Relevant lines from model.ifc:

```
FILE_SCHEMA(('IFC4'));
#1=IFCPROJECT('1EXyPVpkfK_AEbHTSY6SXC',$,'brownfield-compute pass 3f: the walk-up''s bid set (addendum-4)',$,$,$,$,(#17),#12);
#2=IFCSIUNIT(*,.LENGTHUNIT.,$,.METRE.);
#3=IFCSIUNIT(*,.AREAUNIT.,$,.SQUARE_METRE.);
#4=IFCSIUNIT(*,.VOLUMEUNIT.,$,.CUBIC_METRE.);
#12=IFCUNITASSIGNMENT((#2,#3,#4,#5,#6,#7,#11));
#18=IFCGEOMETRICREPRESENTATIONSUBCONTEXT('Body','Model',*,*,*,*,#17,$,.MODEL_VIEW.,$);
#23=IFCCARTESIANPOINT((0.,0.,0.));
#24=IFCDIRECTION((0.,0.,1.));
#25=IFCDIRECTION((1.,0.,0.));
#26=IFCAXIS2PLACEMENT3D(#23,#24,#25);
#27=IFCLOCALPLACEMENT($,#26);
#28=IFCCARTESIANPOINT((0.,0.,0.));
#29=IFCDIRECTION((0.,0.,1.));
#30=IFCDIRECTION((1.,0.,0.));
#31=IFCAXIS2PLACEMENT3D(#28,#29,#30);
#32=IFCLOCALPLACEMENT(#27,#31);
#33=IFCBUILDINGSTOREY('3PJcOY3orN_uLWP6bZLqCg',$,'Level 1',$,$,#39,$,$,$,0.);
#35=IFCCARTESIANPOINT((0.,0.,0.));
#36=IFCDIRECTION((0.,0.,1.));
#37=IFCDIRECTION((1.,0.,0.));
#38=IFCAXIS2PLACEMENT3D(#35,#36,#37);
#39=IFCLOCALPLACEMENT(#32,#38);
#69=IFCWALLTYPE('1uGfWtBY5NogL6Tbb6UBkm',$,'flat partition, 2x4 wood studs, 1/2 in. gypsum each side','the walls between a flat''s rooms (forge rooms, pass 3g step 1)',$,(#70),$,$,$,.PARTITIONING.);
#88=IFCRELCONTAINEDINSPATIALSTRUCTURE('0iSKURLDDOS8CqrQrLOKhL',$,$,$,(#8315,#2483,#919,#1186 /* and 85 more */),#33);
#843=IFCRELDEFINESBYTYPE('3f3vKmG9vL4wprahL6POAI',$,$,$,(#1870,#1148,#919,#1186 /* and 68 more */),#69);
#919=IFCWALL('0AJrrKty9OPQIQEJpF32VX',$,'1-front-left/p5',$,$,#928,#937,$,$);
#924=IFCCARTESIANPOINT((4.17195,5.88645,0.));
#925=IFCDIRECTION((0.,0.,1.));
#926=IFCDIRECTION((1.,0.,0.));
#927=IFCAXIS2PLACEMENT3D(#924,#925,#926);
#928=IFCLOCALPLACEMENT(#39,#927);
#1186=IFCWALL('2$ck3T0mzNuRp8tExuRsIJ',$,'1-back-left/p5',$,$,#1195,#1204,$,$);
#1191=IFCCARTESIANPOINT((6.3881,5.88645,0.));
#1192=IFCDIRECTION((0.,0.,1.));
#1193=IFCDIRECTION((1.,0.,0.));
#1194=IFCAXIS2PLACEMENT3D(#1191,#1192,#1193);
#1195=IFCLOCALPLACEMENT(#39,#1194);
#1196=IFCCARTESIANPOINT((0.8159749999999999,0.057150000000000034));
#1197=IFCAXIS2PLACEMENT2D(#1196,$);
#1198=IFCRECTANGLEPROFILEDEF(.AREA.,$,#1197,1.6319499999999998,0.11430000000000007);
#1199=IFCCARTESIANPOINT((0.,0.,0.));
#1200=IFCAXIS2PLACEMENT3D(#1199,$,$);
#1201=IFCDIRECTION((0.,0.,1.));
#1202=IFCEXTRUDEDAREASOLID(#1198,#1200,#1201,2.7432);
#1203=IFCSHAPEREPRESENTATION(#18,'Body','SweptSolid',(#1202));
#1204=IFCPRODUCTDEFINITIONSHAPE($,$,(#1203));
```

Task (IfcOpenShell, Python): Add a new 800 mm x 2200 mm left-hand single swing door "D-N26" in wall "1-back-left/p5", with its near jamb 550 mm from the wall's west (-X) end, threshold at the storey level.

```python
import numpy as np
import ifcopenshell
import ifcopenshell.api.feature
import ifcopenshell.api.geometry
import ifcopenshell.api.root
import ifcopenshell.api.spatial
import ifcopenshell.geom
import ifcopenshell.util.element
import ifcopenshell.util.placement
import ifcopenshell.util.representation
import ifcopenshell.util.shape
import ifcopenshell.util.unit

model = ifcopenshell.open("model.ifc")
unit_scale = ifcopenshell.util.unit.calculate_unit_scale(model)
settings = ifcopenshell.geom.settings()


def volume(element):
    """Net volume in cubic metres, openings subtracted."""
    shape = ifcopenshell.geom.create_shape(settings, element)
    return ifcopenshell.util.shape.get_volume(shape.geometry)


wall = model.by_id(1186)
storey = ifcopenshell.util.element.get_container(wall, ifc_class="IfcBuildingStorey")
context = ifcopenshell.util.representation.get_context(model, "Model", "Body", "MODEL_VIEW")
before = volume(wall)

width, height, from_end, sill = 0.8, 2.2, 0.55, 0.0  # metres

# The wall runs along its own X axis, and the end named is its -X end.
wall_shape = ifcopenshell.geom.create_shape(settings, wall)
x, y, z = ifcopenshell.util.shape.get_vertices(wall_shape.geometry).T
start = x.min() + from_end
face, thickness = float(y.min()), float(y.max() - y.min())
wall_matrix = ifcopenshell.util.placement.get_local_placement(wall.ObjectPlacement)
level = ifcopenshell.util.placement.get_local_placement(storey.ObjectPlacement)[2, 3]


def in_wall(x, y):
    """Placement at x, y metres in the wall's axes, at sill height."""
    matrix = wall_matrix.copy()
    matrix[:, 3] = wall_matrix @ np.array([x / unit_scale, y / unit_scale, 0.0, 1.0])
    matrix[2, 3] = level + sill / unit_scale
    return matrix


# Opening: a box that overshoots both wall faces by 50 mm.
opening = ifcopenshell.api.root.create_entity(model, ifc_class="IfcOpeningElement", predefined_type="OPENING")
box = ifcopenshell.api.geometry.add_wall_representation(
    model, context=context, length=width, height=height, thickness=thickness + 0.1
)
ifcopenshell.api.geometry.assign_representation(model, product=opening, representation=box)
ifcopenshell.api.geometry.edit_object_placement(model, product=opening, matrix=in_wall(start, face - 0.05), is_si=False)
ifcopenshell.api.feature.add_feature(model, feature=opening, element=wall)

door = ifcopenshell.api.root.create_entity(model, ifc_class="IfcDoor", name="D-N26", predefined_type="DOOR")
door.OverallWidth, door.OverallHeight = width / unit_scale, height / unit_scale
door.OperationType = "SINGLE_SWING_LEFT"
body = ifcopenshell.api.geometry.add_door_representation(
    model,
    context=context,
    overall_width=door.OverallWidth,
    overall_height=door.OverallHeight,
    operation_type="SINGLE_SWING_LEFT",
    lining_properties={"LiningDepth": thickness / unit_scale, "ThresholdDepth": thickness / unit_scale},
)
ifcopenshell.api.geometry.assign_representation(model, product=door, representation=body)
ifcopenshell.api.spatial.assign_container(model, products=[door], relating_structure=storey)
ifcopenshell.api.feature.add_filling(model, opening=opening, element=door)

# The lining spans the wall, so the door starts at the wall face.
ifcopenshell.api.geometry.edit_object_placement(model, product=door, matrix=in_wall(start, face), is_si=False)

after = volume(wall)

print(f"wall volume {before:.3f} -> {after:.3f} m3")

model.write("model_edited.ifc")
```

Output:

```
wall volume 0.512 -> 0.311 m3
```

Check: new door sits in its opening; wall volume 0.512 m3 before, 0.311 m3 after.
